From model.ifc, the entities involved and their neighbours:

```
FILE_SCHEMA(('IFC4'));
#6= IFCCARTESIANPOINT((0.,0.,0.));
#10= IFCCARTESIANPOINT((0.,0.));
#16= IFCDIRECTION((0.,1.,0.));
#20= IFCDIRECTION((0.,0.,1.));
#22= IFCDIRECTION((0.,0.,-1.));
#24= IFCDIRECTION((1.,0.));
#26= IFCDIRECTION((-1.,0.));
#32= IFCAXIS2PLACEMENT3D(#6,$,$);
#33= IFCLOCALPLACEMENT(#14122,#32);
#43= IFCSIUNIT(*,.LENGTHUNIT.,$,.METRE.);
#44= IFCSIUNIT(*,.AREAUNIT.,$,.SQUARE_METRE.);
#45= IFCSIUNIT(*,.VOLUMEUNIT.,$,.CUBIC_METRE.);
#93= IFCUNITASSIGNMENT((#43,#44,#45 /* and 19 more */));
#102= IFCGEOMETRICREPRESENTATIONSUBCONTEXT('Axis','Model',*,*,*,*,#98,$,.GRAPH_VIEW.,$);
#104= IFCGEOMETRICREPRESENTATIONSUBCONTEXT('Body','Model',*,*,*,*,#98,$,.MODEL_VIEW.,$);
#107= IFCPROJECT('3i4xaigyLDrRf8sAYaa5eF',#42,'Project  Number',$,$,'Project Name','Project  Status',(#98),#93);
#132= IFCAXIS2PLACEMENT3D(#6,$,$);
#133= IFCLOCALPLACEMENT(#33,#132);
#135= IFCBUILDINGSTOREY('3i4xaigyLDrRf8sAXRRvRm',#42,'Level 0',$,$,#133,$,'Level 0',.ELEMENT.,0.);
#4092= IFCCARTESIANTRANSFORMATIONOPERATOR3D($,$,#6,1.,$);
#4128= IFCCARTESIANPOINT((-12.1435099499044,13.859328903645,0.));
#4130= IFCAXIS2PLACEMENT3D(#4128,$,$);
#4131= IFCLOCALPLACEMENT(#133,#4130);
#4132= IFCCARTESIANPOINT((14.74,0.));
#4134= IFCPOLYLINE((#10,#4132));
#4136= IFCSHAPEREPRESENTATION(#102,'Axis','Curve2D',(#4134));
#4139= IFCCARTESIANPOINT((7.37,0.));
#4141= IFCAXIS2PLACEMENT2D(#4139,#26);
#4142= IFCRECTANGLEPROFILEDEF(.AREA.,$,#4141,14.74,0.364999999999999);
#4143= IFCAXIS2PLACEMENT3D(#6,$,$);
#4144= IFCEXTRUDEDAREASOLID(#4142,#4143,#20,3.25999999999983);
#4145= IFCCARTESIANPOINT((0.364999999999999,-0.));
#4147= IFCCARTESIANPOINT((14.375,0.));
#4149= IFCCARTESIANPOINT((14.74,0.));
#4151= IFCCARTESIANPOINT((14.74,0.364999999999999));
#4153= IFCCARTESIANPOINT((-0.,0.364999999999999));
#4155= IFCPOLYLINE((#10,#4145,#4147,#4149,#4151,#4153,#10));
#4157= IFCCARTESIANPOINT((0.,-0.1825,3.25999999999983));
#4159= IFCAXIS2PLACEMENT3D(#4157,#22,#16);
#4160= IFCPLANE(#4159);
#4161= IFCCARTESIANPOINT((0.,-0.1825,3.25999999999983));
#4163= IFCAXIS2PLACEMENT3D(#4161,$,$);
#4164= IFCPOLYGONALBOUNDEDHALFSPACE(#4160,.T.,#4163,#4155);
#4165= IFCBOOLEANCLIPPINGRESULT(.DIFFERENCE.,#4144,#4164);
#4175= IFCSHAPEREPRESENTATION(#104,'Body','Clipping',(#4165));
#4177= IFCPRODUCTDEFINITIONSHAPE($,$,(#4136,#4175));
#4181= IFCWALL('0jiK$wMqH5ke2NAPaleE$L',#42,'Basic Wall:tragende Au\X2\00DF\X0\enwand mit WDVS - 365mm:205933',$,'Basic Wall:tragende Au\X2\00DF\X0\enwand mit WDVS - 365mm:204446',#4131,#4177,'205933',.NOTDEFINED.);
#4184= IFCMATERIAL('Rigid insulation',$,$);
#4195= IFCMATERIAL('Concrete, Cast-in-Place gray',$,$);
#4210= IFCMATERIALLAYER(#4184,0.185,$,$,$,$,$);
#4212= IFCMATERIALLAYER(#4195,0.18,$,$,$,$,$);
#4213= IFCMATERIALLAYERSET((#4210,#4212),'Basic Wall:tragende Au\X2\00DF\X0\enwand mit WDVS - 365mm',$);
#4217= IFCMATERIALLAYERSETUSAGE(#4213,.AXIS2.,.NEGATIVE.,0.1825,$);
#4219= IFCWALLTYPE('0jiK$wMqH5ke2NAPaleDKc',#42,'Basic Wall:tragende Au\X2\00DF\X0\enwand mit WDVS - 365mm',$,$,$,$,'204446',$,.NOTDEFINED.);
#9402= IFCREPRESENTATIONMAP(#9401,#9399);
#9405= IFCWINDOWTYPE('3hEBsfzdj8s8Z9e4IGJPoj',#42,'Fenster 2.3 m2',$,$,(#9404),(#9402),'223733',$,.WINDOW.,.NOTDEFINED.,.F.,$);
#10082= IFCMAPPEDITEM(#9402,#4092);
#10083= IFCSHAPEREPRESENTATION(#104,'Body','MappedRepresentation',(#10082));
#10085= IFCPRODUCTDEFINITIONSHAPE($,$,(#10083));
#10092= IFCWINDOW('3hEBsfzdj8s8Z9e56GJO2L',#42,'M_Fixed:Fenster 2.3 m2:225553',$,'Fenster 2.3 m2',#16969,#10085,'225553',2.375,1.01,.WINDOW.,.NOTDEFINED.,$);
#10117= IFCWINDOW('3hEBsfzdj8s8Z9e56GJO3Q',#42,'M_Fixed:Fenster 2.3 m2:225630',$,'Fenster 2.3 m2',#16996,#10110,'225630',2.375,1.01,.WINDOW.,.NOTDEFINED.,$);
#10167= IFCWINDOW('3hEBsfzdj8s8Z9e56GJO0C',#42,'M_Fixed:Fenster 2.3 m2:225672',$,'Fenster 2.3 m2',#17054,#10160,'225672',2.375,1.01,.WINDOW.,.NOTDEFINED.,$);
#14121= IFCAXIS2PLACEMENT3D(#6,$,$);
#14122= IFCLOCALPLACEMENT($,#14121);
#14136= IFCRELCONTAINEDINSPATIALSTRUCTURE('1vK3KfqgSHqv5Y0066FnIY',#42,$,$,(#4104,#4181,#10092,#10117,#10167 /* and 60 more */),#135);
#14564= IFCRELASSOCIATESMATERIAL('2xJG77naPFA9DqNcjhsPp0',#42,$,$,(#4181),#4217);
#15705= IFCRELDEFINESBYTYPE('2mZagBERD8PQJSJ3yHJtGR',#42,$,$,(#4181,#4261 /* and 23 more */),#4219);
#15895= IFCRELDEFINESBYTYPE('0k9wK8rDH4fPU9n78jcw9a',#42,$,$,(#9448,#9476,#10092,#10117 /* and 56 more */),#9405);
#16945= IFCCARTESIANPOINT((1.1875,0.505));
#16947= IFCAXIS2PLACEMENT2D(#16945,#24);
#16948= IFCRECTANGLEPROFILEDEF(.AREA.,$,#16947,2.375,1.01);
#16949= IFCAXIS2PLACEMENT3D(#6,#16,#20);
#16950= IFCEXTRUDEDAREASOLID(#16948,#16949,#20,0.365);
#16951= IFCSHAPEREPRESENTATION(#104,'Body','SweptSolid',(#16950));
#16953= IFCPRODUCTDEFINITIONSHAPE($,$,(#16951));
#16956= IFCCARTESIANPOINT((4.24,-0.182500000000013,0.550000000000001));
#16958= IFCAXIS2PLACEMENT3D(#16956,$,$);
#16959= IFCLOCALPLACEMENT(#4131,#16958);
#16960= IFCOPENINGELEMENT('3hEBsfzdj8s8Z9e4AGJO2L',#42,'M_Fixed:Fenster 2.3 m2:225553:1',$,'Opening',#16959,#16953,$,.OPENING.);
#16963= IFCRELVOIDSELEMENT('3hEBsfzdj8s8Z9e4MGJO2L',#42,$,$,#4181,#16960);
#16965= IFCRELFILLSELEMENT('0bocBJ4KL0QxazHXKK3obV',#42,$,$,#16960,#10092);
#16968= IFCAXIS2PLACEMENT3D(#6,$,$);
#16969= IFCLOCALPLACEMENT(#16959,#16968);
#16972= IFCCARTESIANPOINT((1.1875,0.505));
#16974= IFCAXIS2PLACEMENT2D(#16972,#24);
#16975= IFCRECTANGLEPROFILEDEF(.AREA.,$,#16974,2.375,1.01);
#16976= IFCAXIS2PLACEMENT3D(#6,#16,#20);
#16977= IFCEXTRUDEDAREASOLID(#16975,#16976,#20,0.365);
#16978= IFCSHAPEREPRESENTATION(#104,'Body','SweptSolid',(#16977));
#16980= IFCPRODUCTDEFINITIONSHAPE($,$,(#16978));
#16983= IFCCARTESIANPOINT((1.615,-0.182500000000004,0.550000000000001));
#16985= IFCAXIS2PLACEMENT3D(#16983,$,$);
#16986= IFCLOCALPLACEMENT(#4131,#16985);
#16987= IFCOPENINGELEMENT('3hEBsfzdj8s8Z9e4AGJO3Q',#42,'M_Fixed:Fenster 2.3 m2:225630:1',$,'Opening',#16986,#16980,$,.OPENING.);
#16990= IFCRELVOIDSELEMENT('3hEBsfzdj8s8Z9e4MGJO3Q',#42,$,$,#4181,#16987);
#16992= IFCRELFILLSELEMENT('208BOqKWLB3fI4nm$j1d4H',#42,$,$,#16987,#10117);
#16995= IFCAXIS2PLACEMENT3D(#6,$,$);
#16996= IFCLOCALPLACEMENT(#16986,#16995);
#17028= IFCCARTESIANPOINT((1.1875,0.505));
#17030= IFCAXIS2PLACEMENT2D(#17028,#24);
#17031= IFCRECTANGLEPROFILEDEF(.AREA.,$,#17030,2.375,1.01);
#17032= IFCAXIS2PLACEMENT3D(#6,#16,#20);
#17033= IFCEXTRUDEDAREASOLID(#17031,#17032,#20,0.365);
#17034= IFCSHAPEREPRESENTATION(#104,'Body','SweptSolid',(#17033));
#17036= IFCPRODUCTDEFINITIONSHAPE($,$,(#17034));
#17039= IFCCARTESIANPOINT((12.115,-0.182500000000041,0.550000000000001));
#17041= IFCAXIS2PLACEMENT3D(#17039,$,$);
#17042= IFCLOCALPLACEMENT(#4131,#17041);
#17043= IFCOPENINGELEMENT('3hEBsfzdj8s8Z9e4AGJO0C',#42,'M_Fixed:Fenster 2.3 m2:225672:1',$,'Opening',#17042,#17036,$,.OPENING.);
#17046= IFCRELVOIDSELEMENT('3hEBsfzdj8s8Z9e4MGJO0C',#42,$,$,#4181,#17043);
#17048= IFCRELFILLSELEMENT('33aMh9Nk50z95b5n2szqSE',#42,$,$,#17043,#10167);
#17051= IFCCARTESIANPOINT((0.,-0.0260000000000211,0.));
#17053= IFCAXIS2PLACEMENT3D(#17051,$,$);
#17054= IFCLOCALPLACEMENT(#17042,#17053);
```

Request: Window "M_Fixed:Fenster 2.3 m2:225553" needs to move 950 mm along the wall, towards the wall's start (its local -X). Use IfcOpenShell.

```python
import ifcopenshell
import ifcopenshell.api.geometry
import ifcopenshell.util.placement
import ifcopenshell.util.unit

model = ifcopenshell.open("model.ifc")
unit_scale = ifcopenshell.util.unit.calculate_unit_scale(model)

window = model.by_id(10092)
opening = window.FillsVoids[0].RelatingOpeningElement
wall = opening.VoidsElements[0].RelatingBuildingElement

wall_matrix = ifcopenshell.util.placement.get_local_placement(wall.ObjectPlacement)
shift = wall_matrix[:3, 0] * -0.95 / unit_scale
before = ifcopenshell.util.placement.get_local_placement(window.ObjectPlacement)[:3, 3].copy()

# The window is placed relative to its opening, so it follows when the opening moves.
matrix = ifcopenshell.util.placement.get_local_placement(opening.ObjectPlacement)
matrix[:3, 3] += shift
ifcopenshell.api.geometry.edit_object_placement(
    model, product=opening, matrix=matrix, is_si=False, should_transform_children=True
)

after = ifcopenshell.util.placement.get_local_placement(window.ObjectPlacement)[:3, 3]
print("window moved by", (after - before).round(3) + 0.0)

model.write("model_v2.ifc")
```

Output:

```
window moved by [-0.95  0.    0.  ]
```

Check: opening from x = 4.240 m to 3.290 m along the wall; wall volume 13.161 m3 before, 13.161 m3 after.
